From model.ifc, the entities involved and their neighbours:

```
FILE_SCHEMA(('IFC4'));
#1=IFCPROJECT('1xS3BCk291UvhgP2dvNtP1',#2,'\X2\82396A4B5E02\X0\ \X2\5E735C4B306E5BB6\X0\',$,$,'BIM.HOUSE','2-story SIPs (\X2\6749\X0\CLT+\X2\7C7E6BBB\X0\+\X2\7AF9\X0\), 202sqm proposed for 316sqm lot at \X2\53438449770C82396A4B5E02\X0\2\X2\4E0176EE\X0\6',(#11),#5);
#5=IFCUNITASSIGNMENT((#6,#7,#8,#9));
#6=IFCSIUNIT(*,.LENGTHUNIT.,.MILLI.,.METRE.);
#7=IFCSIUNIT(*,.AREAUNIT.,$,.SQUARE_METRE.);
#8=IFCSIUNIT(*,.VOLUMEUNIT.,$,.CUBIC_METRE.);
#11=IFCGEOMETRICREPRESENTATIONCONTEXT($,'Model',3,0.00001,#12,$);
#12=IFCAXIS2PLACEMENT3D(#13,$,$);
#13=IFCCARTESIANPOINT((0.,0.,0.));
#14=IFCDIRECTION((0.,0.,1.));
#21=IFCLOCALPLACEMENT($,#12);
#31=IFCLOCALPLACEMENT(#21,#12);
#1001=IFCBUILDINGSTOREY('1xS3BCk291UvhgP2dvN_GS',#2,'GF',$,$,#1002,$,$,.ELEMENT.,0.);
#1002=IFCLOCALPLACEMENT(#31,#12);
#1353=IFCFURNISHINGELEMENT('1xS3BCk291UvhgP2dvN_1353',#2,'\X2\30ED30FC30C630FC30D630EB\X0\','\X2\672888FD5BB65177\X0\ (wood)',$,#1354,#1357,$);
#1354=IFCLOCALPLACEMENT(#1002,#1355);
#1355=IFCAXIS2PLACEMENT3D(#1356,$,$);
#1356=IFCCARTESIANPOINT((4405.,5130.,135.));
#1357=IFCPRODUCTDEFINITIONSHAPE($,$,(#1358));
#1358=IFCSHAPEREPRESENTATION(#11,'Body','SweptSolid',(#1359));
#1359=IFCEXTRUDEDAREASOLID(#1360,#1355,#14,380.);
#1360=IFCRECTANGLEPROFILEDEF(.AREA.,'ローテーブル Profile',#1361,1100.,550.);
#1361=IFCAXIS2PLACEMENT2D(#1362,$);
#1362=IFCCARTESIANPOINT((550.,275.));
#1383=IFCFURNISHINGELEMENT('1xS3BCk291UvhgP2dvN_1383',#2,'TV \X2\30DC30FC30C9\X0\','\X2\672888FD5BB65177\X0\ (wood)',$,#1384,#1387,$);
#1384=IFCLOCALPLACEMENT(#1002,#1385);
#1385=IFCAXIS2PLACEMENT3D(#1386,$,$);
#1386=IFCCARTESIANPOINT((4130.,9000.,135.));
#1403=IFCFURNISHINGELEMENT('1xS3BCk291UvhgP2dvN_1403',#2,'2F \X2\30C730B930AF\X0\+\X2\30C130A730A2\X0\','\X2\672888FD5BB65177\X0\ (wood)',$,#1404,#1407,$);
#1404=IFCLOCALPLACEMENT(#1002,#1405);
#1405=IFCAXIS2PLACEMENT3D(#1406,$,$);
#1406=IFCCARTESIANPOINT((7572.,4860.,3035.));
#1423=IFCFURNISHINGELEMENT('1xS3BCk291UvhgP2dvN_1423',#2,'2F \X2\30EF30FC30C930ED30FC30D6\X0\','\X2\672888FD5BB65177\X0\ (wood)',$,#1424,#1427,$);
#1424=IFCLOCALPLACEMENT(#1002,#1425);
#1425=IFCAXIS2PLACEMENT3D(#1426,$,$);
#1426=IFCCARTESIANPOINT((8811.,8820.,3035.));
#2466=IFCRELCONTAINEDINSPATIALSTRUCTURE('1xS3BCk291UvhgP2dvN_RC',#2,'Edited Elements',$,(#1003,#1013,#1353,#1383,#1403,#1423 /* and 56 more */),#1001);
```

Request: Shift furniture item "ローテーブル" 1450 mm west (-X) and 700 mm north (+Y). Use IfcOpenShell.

```python
import ifcopenshell
import ifcopenshell.api.geometry
import ifcopenshell.util.placement

model = ifcopenshell.open("model.ifc")

item = model.by_id(1353)
matrix = ifcopenshell.util.placement.get_local_placement(item.ObjectPlacement)
matrix[0, 3] -= 1450.0
matrix[1, 3] += 700.0
ifcopenshell.api.geometry.edit_object_placement(model, product=item, matrix=matrix, is_si=False)

print(ifcopenshell.util.placement.get_local_placement(item.ObjectPlacement).round(3) + 0.0)

model.write("model_edited.ifc")
```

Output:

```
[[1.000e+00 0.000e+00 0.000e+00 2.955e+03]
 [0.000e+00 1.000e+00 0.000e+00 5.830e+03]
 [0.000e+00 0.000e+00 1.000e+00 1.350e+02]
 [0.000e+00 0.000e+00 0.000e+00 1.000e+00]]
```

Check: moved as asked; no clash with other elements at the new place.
